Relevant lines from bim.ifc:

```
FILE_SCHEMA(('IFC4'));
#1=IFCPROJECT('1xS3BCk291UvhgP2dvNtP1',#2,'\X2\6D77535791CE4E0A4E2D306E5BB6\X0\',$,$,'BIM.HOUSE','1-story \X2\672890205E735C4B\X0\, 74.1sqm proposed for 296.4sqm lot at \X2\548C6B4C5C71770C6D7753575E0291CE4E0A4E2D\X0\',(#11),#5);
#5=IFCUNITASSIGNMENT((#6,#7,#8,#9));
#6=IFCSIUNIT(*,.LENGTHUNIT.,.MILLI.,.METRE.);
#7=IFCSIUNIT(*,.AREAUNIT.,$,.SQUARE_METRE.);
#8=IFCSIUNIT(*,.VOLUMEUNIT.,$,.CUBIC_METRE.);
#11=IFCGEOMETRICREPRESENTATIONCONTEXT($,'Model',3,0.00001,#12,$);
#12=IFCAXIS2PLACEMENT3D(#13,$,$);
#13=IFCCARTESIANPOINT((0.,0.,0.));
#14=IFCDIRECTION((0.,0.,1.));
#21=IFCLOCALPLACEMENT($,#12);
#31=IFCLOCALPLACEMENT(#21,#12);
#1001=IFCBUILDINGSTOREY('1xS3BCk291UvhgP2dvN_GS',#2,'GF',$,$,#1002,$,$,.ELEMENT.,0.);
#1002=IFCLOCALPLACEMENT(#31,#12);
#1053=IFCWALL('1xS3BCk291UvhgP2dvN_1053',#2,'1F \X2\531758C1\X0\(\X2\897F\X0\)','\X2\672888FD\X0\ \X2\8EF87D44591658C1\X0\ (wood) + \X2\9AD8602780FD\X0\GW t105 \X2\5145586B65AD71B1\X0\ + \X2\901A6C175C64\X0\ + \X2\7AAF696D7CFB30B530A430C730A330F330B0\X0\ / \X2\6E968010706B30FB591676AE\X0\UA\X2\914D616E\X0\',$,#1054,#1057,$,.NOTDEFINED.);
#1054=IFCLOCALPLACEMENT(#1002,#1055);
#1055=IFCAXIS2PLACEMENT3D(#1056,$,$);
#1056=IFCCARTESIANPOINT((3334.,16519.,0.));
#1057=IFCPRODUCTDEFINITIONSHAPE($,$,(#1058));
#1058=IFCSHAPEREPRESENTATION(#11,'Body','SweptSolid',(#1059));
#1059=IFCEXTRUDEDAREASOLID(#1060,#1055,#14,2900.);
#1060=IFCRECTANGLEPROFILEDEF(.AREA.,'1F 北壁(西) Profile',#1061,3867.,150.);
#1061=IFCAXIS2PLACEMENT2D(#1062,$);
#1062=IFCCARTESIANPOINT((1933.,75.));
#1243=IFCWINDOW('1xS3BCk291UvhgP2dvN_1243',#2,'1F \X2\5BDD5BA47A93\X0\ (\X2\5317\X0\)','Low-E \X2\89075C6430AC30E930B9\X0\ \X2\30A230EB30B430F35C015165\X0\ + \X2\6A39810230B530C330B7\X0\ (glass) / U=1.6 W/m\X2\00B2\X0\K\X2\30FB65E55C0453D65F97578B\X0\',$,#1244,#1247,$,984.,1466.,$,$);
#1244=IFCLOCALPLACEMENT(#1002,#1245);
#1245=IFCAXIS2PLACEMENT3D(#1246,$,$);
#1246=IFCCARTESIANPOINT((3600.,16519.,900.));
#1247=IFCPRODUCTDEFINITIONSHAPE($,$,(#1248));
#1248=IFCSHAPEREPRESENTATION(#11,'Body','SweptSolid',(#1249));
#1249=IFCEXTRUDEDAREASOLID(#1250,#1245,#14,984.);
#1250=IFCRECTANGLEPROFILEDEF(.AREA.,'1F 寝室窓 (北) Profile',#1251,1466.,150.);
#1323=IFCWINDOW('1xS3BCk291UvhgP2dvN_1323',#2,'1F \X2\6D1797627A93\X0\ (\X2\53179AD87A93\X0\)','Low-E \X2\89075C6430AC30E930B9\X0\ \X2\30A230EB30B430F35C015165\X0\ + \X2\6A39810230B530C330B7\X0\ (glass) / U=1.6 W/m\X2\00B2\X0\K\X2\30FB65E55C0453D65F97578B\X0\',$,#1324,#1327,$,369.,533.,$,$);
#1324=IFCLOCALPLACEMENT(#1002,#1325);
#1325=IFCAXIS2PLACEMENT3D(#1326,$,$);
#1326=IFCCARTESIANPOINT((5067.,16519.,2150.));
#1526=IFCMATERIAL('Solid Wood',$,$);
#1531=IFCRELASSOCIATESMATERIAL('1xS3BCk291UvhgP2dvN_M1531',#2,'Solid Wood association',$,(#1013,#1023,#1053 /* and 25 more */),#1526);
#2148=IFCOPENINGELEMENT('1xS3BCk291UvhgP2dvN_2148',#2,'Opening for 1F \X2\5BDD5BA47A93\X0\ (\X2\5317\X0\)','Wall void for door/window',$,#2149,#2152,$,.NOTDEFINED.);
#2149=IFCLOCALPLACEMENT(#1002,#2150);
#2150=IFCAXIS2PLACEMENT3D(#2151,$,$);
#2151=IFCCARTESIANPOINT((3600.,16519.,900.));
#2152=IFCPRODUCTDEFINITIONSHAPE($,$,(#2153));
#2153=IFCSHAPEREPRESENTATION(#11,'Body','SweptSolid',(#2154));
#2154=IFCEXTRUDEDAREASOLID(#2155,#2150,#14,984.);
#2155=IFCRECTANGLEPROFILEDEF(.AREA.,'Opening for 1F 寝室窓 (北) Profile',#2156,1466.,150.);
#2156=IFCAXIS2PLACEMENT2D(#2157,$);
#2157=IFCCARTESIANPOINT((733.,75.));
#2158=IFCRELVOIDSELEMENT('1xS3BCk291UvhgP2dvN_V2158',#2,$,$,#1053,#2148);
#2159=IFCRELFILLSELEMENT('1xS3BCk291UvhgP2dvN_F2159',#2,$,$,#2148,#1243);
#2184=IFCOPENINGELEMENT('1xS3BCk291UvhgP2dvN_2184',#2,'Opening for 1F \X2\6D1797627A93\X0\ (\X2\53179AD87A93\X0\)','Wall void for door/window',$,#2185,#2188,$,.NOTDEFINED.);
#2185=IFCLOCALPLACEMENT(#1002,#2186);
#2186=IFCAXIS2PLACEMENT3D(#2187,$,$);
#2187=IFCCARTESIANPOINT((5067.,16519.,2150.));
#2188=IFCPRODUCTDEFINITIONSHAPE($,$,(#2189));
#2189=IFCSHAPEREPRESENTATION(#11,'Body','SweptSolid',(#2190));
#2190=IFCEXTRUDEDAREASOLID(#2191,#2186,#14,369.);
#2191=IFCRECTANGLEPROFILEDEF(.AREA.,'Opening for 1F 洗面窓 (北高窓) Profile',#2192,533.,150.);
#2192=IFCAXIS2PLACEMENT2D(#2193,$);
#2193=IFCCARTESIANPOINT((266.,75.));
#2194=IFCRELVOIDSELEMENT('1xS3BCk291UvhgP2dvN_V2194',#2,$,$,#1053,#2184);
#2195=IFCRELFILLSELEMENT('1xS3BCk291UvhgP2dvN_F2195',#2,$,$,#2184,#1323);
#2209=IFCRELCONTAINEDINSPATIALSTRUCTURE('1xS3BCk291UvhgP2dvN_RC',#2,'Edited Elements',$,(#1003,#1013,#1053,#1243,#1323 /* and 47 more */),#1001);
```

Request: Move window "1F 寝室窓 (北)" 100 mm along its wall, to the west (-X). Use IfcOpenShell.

```python
import ifcopenshell
import ifcopenshell.api.geometry
import ifcopenshell.util.placement

model = ifcopenshell.open("bim.ifc")

window = model.by_guid("1xS3BCk291UvhgP2dvN_1243")
opening = window.FillsVoids[0].RelatingOpeningElement
wall = opening.VoidsElements[0].RelatingBuildingElement

wall_matrix = ifcopenshell.util.placement.get_local_placement(wall.ObjectPlacement)
shift = wall_matrix[:3, 0] * -100.0
before = ifcopenshell.util.placement.get_local_placement(window.ObjectPlacement)[:3, 3].copy()

# The window is not placed relative to its opening, so move both.
for product in (opening, window):
    matrix = ifcopenshell.util.placement.get_local_placement(product.ObjectPlacement)
    matrix[:3, 3] += shift
    ifcopenshell.api.geometry.edit_object_placement(model, product=product, matrix=matrix, is_si=False)

after = ifcopenshell.util.placement.get_local_placement(window.ObjectPlacement)[:3, 3]
print("window moved by", (after - before).round(3) + 0.0)

model.write("bim-out.ifc")
```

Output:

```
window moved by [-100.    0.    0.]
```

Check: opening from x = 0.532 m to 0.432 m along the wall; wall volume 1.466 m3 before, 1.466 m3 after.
